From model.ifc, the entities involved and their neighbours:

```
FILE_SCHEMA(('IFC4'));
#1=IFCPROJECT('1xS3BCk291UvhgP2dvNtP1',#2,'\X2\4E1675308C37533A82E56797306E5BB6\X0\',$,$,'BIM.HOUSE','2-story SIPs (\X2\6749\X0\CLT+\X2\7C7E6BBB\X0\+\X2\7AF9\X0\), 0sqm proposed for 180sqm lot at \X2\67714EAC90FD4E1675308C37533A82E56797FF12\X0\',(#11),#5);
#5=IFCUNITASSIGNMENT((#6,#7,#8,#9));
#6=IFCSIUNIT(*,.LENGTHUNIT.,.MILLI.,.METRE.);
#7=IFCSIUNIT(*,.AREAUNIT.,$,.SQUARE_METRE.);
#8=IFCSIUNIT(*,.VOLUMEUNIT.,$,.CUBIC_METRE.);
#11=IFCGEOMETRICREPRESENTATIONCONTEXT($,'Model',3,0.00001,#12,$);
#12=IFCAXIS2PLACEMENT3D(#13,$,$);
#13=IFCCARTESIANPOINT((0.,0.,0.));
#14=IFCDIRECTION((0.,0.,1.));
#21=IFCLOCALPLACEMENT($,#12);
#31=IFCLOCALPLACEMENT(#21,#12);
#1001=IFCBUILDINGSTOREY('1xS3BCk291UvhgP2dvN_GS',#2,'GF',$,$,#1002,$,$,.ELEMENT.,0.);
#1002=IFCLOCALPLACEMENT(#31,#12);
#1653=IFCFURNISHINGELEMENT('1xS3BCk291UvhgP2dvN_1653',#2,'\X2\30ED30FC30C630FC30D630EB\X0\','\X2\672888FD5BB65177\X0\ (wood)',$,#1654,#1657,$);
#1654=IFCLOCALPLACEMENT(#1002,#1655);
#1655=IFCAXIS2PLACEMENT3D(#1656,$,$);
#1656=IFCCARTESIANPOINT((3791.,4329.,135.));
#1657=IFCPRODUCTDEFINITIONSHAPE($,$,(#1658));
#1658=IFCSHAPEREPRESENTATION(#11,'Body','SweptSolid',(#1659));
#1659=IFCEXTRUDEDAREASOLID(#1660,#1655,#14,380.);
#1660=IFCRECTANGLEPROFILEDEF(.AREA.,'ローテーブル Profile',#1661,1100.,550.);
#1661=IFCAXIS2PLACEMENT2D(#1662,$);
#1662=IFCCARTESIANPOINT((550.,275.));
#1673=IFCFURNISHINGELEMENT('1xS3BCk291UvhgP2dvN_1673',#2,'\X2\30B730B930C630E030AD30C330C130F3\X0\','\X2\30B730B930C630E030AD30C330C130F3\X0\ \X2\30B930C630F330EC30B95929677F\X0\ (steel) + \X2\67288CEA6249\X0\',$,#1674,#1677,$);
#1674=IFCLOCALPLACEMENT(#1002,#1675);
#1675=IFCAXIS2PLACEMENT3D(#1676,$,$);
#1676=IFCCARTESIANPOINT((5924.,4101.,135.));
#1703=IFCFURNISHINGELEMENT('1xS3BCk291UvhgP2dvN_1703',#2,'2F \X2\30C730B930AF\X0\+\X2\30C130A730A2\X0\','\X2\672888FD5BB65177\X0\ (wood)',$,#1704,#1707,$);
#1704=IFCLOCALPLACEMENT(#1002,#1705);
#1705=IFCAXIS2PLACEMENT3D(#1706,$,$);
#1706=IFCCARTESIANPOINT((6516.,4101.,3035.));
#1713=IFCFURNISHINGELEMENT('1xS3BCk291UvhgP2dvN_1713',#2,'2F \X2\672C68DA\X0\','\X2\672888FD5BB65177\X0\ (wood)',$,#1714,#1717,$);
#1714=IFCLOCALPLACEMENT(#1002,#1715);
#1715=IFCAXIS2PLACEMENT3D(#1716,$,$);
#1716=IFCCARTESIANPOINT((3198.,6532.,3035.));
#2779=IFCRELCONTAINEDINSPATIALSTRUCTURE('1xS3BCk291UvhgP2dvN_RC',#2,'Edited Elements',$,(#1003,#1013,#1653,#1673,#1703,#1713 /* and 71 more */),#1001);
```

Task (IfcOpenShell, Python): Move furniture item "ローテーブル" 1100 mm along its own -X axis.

```python
import ifcopenshell
import ifcopenshell.api.geometry
import ifcopenshell.util.placement
import ifcopenshell.util.unit

model = ifcopenshell.open("model.ifc")
unit_scale = ifcopenshell.util.unit.calculate_unit_scale(model)

item = model.by_guid("1xS3BCk291UvhgP2dvN_1653")
matrix = ifcopenshell.util.placement.get_local_placement(item.ObjectPlacement)
matrix[:3, 3] -= matrix[:3, 0] * 1.1 / unit_scale
ifcopenshell.api.geometry.edit_object_placement(model, product=item, matrix=matrix, is_si=False)

print(ifcopenshell.util.placement.get_local_placement(item.ObjectPlacement).round(3) + 0.0)

model.write("model_updated.ifc")
```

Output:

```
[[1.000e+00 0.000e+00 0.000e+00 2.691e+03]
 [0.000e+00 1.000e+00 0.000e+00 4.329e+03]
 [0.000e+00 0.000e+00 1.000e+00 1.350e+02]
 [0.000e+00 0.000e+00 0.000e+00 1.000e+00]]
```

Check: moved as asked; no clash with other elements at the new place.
